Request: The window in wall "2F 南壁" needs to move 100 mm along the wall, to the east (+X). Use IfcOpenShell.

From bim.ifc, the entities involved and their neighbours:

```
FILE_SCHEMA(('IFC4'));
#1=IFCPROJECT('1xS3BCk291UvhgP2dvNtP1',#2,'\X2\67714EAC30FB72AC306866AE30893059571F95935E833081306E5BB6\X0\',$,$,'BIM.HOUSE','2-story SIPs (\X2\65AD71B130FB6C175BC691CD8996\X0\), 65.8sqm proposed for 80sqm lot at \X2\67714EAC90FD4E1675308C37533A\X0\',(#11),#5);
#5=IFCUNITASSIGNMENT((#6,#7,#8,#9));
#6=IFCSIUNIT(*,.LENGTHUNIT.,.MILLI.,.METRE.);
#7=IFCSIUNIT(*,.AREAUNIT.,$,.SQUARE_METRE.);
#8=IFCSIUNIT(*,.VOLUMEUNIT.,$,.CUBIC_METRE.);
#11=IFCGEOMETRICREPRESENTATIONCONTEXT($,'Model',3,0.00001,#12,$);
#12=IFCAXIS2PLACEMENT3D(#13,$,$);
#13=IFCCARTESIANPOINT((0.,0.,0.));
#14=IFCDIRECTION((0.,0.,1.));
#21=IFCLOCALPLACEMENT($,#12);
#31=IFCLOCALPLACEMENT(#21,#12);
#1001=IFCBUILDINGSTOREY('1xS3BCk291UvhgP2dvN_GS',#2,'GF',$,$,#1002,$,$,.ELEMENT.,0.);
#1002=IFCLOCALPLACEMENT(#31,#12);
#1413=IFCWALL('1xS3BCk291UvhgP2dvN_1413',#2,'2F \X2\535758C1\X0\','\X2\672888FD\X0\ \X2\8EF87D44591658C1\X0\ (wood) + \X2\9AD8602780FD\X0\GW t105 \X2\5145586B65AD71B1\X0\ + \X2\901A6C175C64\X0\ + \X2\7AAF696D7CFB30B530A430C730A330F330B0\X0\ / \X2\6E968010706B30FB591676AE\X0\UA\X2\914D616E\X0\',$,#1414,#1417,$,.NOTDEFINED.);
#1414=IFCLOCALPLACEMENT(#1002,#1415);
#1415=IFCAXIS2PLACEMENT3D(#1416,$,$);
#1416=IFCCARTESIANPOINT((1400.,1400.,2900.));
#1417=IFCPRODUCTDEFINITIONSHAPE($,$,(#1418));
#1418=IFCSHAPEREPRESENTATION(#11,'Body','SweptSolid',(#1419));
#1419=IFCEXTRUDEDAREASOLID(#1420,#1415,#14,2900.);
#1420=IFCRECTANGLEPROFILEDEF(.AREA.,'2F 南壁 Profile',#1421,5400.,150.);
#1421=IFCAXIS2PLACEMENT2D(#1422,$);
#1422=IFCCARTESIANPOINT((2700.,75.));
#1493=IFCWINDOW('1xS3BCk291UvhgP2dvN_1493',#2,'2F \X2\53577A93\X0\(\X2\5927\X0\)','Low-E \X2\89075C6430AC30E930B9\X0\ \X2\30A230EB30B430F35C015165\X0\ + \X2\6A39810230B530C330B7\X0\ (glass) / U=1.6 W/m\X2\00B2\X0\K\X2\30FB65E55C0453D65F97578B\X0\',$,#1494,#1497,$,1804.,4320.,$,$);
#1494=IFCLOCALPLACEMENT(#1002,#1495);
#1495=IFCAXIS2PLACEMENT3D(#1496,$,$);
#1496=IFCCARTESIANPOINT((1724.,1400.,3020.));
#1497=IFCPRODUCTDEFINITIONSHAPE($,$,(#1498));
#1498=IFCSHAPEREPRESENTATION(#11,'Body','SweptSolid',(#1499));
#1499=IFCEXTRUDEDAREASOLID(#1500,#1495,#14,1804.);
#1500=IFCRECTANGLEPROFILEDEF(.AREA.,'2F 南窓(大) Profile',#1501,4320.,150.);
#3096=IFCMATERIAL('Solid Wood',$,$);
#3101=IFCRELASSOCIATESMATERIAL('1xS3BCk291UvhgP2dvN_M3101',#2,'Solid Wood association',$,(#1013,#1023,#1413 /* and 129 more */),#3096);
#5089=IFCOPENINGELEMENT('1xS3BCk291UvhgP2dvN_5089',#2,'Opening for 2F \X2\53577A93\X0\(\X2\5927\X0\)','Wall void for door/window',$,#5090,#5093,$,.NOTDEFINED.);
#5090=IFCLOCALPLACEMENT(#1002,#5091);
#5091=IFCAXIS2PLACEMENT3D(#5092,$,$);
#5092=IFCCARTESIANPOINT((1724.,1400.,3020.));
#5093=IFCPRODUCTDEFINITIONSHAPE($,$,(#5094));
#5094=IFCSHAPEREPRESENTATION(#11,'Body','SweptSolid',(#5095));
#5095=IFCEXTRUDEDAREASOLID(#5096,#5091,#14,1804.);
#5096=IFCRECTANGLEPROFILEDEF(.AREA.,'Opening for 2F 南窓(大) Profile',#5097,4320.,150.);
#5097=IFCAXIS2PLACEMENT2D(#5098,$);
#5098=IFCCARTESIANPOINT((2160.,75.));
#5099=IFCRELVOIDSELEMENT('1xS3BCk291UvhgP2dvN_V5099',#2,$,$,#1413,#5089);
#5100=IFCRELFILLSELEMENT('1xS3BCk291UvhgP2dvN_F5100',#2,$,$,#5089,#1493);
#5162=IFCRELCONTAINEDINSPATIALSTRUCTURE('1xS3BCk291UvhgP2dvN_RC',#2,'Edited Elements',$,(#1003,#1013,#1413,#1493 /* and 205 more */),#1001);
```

```python
import ifcopenshell
import ifcopenshell.api.geometry
import ifcopenshell.util.placement
import ifcopenshell.util.unit

model = ifcopenshell.open("bim.ifc")
unit_scale = ifcopenshell.util.unit.calculate_unit_scale(model)

window = model.by_guid("1xS3BCk291UvhgP2dvN_1493")
opening = window.FillsVoids[0].RelatingOpeningElement
wall = opening.VoidsElements[0].RelatingBuildingElement

wall_matrix = ifcopenshell.util.placement.get_local_placement(wall.ObjectPlacement)
shift = wall_matrix[:3, 0] * 0.1 / unit_scale
before = ifcopenshell.util.placement.get_local_placement(window.ObjectPlacement)[:3, 3].copy()

# The window is not placed relative to its opening, so move both.
for product in (opening, window):
    matrix = ifcopenshell.util.placement.get_local_placement(product.ObjectPlacement)
    matrix[:3, 3] += shift
    ifcopenshell.api.geometry.edit_object_placement(model, product=product, matrix=matrix, is_si=False)

after = ifcopenshell.util.placement.get_local_placement(window.ObjectPlacement)[:3, 3]
print("window moved by", (after - before).round(3) + 0.0)

model.write("bim-out.ifc")
```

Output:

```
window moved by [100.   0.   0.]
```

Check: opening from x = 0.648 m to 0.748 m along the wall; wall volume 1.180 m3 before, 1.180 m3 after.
